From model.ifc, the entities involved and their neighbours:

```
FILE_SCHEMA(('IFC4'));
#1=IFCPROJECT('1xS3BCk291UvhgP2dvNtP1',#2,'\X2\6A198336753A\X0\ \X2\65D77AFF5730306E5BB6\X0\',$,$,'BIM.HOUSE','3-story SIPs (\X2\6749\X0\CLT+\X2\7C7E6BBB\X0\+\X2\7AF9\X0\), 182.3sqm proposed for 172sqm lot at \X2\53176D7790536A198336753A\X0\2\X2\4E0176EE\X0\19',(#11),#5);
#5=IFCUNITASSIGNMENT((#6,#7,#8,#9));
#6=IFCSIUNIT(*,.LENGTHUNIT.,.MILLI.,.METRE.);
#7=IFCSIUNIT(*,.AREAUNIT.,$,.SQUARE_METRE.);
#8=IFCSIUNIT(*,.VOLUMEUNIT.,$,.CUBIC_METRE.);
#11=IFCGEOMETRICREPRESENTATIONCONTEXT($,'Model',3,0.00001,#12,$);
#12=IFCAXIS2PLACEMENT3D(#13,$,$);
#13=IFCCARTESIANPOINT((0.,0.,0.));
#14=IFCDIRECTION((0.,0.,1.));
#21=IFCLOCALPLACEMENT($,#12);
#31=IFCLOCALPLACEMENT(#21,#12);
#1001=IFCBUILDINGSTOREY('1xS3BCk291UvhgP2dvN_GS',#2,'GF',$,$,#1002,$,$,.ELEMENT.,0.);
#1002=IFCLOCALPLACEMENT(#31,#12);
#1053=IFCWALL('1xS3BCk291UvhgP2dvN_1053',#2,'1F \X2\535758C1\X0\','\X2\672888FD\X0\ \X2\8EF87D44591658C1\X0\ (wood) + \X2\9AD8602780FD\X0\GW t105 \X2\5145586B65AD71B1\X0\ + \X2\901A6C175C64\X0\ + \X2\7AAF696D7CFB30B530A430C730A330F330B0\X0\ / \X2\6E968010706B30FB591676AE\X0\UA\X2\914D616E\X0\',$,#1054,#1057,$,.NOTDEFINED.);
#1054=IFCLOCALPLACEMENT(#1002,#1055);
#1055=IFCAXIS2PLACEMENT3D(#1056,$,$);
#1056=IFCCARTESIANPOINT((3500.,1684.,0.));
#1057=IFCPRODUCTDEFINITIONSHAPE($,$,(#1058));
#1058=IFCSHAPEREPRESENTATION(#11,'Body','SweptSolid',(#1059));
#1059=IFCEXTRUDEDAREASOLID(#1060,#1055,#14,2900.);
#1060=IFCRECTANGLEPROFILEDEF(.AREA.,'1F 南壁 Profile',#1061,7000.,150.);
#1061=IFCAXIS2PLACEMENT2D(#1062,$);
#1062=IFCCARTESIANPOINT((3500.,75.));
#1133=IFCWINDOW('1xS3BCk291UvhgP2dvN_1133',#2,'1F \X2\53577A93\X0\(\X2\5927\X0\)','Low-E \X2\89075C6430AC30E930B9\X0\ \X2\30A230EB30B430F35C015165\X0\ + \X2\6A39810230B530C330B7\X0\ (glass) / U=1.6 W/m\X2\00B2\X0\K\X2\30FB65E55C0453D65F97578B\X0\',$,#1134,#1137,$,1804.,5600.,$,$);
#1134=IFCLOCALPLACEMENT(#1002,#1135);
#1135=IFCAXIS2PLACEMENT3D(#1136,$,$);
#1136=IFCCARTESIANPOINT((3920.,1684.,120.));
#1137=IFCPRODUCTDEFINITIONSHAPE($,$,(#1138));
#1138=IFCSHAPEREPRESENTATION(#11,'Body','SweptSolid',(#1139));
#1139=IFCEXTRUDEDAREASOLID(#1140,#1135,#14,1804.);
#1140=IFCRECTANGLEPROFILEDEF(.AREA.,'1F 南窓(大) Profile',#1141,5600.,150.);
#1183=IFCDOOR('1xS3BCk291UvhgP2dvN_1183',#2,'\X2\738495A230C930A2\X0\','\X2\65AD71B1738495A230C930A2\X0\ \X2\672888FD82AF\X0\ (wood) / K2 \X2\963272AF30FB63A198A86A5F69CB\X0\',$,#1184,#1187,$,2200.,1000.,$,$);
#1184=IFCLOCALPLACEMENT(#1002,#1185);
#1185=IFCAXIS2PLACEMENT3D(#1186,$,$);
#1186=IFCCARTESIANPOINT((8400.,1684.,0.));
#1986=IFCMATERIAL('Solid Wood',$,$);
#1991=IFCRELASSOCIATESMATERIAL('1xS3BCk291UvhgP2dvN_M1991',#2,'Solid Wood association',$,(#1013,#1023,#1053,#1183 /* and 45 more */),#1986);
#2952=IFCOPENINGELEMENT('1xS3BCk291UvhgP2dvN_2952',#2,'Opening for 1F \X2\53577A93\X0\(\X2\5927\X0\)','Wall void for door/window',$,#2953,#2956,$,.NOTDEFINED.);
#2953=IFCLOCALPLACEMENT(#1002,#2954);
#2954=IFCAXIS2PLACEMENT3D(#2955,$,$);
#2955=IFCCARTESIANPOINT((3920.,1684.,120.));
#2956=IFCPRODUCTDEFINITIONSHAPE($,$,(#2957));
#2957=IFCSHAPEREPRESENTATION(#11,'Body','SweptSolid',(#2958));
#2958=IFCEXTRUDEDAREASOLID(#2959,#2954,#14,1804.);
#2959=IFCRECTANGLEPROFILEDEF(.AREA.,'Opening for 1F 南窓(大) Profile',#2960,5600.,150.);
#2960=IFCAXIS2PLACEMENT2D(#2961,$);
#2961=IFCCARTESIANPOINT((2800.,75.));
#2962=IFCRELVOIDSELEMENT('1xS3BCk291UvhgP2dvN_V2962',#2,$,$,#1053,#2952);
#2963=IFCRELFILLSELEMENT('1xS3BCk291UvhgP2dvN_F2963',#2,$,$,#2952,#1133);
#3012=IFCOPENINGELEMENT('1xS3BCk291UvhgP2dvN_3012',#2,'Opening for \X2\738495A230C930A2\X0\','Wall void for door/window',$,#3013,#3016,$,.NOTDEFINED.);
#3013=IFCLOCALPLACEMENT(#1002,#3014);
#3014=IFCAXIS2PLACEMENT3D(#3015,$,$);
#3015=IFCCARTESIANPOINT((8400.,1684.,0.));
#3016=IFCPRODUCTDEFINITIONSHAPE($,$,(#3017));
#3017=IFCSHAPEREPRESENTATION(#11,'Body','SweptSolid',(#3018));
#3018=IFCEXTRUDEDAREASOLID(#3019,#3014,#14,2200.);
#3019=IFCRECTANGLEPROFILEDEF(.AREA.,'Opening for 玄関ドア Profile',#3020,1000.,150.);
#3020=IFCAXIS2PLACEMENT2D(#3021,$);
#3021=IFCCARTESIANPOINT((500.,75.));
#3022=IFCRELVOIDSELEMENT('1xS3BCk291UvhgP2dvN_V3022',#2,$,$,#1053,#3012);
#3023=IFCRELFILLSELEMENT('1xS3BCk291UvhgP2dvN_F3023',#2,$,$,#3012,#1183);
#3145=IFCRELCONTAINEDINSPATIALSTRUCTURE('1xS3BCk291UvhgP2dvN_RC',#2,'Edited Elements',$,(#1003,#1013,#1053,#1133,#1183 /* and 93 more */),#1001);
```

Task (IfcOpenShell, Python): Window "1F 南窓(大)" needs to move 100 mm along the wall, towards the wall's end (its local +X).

```python
import ifcopenshell
import ifcopenshell.api.geometry
import ifcopenshell.util.placement

model = ifcopenshell.open("model.ifc")

window = model.by_id(1133)
opening = window.FillsVoids[0].RelatingOpeningElement
wall = opening.VoidsElements[0].RelatingBuildingElement

wall_matrix = ifcopenshell.util.placement.get_local_placement(wall.ObjectPlacement)
shift = wall_matrix[:3, 0] * 100.0
before = ifcopenshell.util.placement.get_local_placement(window.ObjectPlacement)[:3, 3].copy()

# The window is not placed relative to its opening, so move both.
for product in (opening, window):
    matrix = ifcopenshell.util.placement.get_local_placement(product.ObjectPlacement)
    matrix[:3, 3] += shift
    ifcopenshell.api.geometry.edit_object_placement(model, product=product, matrix=matrix, is_si=False)

after = ifcopenshell.util.placement.get_local_placement(window.ObjectPlacement)[:3, 3]
print("window moved by", (after - before).round(3) + 0.0)

model.write("model_edited.ifc")
```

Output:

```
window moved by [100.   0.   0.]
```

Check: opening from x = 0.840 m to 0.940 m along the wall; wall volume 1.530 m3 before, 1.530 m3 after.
